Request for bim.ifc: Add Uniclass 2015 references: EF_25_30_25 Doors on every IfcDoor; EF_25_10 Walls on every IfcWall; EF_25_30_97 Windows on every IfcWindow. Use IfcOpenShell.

First a look at what the model holds.

```python
import ifcopenshell

model = ifcopenshell.open("bim.ifc")
print(model.schema)
print("classifications:", [c.Name for c in model.by_type("IfcClassification")])
for ifc_class in ("IfcDoor", "IfcRoof", "IfcStair", "IfcWall", "IfcWindow"):
    print(ifc_class, len(model.by_type(ifc_class)))
```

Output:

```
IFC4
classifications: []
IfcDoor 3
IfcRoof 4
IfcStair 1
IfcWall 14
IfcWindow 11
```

```python
import ifcopenshell
import ifcopenshell.api.classification

model = ifcopenshell.open("bim.ifc")

system = ifcopenshell.api.classification.add_classification(model, classification="Uniclass 2015")

codes = {
    "IfcDoor": ("EF_25_30_25", "Doors"),
    "IfcWall": ("EF_25_10", "Walls"),
    "IfcWindow": ("EF_25_30_97", "Windows"),
}
for ifc_class, (code, name) in codes.items():
    products = model.by_type(ifc_class)
    ifcopenshell.api.classification.add_reference(
        model, products=products, classification=system, identification=code, name=name
    )
    print(code, len(products))

model.write("bim_updated.ifc")
```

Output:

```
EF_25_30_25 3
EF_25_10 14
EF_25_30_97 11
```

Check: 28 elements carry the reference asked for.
